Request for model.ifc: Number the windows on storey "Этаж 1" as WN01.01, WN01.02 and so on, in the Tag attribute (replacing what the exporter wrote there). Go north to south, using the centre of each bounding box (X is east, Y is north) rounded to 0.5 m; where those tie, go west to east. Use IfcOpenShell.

First a look at what the model holds.

```python
import ifcopenshell
import ifcopenshell.util.element
import ifcopenshell.util.placement

model = ifcopenshell.open("model.ifc")
print(model.schema)
storey = next(s for s in model.by_type("IfcBuildingStorey") if s.Name == "Этаж 1")
windows = [e for e in ifcopenshell.util.element.get_decomposition(storey) if e.is_a("IfcWindow")]
for e in sorted(windows, key=lambda e: e.id()):
    origin = ifcopenshell.util.placement.get_local_placement(e.ObjectPlacement)[:3, 3]
    print(e.id(), e.Tag, e.Name, origin.round(2) + 0.0, sep=" | ")
```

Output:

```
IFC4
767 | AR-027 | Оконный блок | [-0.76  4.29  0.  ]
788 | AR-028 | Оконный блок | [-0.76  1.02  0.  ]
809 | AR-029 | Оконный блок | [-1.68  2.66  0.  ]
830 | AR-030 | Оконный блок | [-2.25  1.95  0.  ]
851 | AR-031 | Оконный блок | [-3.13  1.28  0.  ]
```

```python
import ifcopenshell
import ifcopenshell.geom
import ifcopenshell.util.element
import ifcopenshell.util.shape

model = ifcopenshell.open("model.ifc")
settings = ifcopenshell.geom.settings()
settings.set("use-world-coords", True)


def centre(element):
    shape = ifcopenshell.geom.create_shape(settings, element)
    return ifcopenshell.util.shape.get_bbox_centroid(shape.geometry)


storey = next(s for s in model.by_type("IfcBuildingStorey") if s.Name == "Этаж 1")
windows = [e for e in ifcopenshell.util.element.get_decomposition(storey) if e.is_a("IfcWindow")]

# Insertion points can sit at a corner or the storey origin, so sort by the geometry (in metres).
centres = {e: centre(e) for e in windows}
windows.sort(key=lambda e: (-round(centres[e][1] / 0.5), centres[e][0]))

for i, e in enumerate(windows, start=1):
    number = f"WN01.{i:02d}"
    e.Tag = number
    print(e.id(), number)

model.write("model_updated.ifc")
```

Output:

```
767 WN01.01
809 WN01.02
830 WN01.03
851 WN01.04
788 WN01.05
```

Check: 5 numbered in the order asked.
